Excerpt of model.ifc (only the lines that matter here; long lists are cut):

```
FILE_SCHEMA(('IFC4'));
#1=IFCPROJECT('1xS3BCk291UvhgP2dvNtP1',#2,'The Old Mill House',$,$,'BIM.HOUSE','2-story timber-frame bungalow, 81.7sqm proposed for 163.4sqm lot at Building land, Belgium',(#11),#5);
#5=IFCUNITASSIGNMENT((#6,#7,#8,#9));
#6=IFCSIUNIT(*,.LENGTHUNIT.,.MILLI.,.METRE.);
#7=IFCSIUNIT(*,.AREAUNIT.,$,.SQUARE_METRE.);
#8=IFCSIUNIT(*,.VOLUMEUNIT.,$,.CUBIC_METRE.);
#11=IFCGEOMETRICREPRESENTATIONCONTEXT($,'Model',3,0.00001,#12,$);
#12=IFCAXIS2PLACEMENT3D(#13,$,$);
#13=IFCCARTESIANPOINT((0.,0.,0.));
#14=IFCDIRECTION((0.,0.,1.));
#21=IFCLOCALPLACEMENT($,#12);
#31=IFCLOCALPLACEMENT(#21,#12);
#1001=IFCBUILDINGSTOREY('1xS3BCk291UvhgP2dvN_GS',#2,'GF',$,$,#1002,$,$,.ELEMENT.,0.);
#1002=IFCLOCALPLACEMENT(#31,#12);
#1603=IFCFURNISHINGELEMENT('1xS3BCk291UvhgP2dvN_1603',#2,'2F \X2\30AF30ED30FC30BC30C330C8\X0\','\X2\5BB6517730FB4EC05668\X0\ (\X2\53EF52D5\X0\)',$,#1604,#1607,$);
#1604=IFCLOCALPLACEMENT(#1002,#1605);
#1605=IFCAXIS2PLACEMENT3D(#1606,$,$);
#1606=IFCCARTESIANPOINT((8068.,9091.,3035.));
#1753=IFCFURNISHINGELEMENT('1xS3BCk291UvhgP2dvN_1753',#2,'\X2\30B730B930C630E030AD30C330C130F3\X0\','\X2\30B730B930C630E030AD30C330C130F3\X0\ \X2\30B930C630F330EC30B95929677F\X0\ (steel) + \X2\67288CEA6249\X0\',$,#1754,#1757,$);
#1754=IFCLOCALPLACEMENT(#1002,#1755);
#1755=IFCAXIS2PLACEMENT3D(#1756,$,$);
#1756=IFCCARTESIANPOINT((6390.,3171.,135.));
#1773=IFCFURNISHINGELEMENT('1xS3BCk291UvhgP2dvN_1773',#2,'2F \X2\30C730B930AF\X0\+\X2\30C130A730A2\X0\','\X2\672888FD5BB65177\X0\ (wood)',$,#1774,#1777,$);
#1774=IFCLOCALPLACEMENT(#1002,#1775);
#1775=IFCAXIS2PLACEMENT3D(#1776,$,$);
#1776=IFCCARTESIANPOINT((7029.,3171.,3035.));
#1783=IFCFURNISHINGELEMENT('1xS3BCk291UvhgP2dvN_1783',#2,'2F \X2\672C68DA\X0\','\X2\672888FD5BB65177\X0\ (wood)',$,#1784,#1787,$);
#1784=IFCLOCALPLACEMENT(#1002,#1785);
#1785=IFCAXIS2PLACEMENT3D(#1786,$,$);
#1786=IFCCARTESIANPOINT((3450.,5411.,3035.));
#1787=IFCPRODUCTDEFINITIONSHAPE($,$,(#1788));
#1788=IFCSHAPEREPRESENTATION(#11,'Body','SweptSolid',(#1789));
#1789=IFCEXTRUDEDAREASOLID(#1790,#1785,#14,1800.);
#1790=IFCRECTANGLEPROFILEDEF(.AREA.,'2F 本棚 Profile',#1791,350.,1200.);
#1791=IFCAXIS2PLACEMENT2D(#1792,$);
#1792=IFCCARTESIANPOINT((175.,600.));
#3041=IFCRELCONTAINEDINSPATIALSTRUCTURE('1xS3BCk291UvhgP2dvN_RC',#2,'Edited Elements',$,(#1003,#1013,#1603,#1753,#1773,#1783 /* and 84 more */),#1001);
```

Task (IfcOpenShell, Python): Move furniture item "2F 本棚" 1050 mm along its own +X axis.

```python
import ifcopenshell
import ifcopenshell.api.geometry
import ifcopenshell.util.placement
import ifcopenshell.util.unit

model = ifcopenshell.open("model.ifc")
unit_scale = ifcopenshell.util.unit.calculate_unit_scale(model)

item = model.by_id(1783)
matrix = ifcopenshell.util.placement.get_local_placement(item.ObjectPlacement)
matrix[:3, 3] += matrix[:3, 0] * 1.05 / unit_scale
ifcopenshell.api.geometry.edit_object_placement(model, product=item, matrix=matrix, is_si=False)

print(ifcopenshell.util.placement.get_local_placement(item.ObjectPlacement).round(3) + 0.0)

model.write("model-out.ifc")
```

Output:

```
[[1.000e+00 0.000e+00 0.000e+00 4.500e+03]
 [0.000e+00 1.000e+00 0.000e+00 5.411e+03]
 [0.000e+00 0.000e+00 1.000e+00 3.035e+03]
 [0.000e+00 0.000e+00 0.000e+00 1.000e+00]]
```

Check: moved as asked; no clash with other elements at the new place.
